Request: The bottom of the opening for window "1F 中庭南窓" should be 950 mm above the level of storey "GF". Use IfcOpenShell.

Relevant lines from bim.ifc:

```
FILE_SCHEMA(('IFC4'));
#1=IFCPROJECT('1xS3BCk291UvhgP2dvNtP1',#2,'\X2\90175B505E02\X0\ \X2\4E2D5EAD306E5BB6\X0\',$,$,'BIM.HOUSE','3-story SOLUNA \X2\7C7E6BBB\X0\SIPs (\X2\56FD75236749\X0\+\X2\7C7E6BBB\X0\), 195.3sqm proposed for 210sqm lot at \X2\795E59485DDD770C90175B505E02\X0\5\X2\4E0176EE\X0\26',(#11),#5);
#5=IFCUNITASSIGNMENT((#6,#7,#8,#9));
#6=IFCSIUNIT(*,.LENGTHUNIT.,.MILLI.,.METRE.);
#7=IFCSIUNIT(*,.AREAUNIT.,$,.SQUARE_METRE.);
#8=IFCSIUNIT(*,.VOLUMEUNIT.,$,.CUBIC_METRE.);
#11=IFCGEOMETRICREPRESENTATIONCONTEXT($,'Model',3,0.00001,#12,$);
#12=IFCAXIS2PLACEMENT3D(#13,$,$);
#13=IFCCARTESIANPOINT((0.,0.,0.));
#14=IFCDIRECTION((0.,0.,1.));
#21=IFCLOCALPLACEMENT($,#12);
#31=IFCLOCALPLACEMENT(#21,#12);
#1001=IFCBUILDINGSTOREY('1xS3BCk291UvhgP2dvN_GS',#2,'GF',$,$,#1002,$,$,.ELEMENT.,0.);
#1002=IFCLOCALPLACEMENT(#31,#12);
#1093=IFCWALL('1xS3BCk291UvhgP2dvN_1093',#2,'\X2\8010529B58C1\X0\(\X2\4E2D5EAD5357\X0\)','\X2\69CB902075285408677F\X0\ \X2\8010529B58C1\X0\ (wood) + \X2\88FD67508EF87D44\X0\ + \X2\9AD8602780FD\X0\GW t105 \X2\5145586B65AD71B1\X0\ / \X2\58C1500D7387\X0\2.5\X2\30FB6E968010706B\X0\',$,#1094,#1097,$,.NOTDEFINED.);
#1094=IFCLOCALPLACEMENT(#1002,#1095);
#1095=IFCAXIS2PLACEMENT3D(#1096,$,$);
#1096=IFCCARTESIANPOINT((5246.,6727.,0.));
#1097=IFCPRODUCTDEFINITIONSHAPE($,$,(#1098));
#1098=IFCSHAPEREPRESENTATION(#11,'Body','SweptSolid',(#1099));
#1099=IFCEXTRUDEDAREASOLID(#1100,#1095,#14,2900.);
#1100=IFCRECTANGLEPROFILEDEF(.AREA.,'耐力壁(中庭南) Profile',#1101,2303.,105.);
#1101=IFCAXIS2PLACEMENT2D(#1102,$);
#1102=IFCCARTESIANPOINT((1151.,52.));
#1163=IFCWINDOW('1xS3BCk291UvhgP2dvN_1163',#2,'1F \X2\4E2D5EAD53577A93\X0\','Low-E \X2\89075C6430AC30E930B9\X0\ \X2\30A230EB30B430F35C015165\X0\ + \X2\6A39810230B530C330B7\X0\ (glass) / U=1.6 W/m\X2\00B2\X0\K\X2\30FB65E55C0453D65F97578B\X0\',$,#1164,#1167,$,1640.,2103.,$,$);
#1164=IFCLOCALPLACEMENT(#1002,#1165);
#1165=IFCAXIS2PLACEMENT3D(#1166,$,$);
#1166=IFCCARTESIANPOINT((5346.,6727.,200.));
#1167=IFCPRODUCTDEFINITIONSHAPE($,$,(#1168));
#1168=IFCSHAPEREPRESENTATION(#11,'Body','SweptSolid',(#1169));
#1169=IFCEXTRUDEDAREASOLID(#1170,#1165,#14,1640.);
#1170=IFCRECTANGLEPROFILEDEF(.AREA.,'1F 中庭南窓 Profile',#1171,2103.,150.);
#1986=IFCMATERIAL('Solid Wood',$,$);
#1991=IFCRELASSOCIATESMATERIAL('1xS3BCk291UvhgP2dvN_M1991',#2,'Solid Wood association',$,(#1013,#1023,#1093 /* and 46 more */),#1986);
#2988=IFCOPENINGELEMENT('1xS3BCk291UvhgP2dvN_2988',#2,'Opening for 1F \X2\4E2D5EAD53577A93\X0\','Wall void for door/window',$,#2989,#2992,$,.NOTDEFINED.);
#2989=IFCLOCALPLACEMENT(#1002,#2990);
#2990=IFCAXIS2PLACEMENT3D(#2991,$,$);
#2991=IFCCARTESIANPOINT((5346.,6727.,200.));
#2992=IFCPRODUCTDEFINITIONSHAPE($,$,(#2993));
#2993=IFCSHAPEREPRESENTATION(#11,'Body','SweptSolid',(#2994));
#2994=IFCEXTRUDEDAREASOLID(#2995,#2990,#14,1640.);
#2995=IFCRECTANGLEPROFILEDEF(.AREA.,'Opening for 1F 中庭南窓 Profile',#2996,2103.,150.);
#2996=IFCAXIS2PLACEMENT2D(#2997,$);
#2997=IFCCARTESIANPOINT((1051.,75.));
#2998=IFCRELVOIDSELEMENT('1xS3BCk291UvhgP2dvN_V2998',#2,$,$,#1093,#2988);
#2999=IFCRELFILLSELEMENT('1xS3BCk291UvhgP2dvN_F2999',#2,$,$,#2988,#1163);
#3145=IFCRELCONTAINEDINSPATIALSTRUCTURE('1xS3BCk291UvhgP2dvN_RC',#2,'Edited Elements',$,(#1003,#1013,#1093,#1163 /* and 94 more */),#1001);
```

```python
import numpy as np
import ifcopenshell
import ifcopenshell.api.geometry
import ifcopenshell.geom
import ifcopenshell.util.element
import ifcopenshell.util.placement
import ifcopenshell.util.shape
import ifcopenshell.util.unit

model = ifcopenshell.open("bim.ifc")
unit_scale = ifcopenshell.util.unit.calculate_unit_scale(model)

window = model.by_guid("1xS3BCk291UvhgP2dvN_1163")
opening = window.FillsVoids[0].RelatingOpeningElement
storey = ifcopenshell.util.element.get_container(window, ifc_class="IfcBuildingStorey")
level = ifcopenshell.util.placement.get_local_placement(storey.ObjectPlacement)[2, 3]

# The opening's origin need not be at the sill, so measure its lowest point.
shape = ifcopenshell.geom.create_shape(ifcopenshell.geom.settings(), opening)
bottom = ifcopenshell.util.shape.get_shape_bottom_elevation(shape, shape.geometry) / unit_scale
dz = level + 0.95 / unit_scale - bottom

shift = np.array([0.0, 0.0, dz])
# The window is not placed relative to its opening, so move both.
for product in (opening, window):
    matrix = ifcopenshell.util.placement.get_local_placement(product.ObjectPlacement)
    matrix[:3, 3] += shift
    ifcopenshell.api.geometry.edit_object_placement(model, product=product, matrix=matrix, is_si=False)

print(f"moved by {dz * unit_scale:+.3f} m")

model.write("bim_edited.ifc")
```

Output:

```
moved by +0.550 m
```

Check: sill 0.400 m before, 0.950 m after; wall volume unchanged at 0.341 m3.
